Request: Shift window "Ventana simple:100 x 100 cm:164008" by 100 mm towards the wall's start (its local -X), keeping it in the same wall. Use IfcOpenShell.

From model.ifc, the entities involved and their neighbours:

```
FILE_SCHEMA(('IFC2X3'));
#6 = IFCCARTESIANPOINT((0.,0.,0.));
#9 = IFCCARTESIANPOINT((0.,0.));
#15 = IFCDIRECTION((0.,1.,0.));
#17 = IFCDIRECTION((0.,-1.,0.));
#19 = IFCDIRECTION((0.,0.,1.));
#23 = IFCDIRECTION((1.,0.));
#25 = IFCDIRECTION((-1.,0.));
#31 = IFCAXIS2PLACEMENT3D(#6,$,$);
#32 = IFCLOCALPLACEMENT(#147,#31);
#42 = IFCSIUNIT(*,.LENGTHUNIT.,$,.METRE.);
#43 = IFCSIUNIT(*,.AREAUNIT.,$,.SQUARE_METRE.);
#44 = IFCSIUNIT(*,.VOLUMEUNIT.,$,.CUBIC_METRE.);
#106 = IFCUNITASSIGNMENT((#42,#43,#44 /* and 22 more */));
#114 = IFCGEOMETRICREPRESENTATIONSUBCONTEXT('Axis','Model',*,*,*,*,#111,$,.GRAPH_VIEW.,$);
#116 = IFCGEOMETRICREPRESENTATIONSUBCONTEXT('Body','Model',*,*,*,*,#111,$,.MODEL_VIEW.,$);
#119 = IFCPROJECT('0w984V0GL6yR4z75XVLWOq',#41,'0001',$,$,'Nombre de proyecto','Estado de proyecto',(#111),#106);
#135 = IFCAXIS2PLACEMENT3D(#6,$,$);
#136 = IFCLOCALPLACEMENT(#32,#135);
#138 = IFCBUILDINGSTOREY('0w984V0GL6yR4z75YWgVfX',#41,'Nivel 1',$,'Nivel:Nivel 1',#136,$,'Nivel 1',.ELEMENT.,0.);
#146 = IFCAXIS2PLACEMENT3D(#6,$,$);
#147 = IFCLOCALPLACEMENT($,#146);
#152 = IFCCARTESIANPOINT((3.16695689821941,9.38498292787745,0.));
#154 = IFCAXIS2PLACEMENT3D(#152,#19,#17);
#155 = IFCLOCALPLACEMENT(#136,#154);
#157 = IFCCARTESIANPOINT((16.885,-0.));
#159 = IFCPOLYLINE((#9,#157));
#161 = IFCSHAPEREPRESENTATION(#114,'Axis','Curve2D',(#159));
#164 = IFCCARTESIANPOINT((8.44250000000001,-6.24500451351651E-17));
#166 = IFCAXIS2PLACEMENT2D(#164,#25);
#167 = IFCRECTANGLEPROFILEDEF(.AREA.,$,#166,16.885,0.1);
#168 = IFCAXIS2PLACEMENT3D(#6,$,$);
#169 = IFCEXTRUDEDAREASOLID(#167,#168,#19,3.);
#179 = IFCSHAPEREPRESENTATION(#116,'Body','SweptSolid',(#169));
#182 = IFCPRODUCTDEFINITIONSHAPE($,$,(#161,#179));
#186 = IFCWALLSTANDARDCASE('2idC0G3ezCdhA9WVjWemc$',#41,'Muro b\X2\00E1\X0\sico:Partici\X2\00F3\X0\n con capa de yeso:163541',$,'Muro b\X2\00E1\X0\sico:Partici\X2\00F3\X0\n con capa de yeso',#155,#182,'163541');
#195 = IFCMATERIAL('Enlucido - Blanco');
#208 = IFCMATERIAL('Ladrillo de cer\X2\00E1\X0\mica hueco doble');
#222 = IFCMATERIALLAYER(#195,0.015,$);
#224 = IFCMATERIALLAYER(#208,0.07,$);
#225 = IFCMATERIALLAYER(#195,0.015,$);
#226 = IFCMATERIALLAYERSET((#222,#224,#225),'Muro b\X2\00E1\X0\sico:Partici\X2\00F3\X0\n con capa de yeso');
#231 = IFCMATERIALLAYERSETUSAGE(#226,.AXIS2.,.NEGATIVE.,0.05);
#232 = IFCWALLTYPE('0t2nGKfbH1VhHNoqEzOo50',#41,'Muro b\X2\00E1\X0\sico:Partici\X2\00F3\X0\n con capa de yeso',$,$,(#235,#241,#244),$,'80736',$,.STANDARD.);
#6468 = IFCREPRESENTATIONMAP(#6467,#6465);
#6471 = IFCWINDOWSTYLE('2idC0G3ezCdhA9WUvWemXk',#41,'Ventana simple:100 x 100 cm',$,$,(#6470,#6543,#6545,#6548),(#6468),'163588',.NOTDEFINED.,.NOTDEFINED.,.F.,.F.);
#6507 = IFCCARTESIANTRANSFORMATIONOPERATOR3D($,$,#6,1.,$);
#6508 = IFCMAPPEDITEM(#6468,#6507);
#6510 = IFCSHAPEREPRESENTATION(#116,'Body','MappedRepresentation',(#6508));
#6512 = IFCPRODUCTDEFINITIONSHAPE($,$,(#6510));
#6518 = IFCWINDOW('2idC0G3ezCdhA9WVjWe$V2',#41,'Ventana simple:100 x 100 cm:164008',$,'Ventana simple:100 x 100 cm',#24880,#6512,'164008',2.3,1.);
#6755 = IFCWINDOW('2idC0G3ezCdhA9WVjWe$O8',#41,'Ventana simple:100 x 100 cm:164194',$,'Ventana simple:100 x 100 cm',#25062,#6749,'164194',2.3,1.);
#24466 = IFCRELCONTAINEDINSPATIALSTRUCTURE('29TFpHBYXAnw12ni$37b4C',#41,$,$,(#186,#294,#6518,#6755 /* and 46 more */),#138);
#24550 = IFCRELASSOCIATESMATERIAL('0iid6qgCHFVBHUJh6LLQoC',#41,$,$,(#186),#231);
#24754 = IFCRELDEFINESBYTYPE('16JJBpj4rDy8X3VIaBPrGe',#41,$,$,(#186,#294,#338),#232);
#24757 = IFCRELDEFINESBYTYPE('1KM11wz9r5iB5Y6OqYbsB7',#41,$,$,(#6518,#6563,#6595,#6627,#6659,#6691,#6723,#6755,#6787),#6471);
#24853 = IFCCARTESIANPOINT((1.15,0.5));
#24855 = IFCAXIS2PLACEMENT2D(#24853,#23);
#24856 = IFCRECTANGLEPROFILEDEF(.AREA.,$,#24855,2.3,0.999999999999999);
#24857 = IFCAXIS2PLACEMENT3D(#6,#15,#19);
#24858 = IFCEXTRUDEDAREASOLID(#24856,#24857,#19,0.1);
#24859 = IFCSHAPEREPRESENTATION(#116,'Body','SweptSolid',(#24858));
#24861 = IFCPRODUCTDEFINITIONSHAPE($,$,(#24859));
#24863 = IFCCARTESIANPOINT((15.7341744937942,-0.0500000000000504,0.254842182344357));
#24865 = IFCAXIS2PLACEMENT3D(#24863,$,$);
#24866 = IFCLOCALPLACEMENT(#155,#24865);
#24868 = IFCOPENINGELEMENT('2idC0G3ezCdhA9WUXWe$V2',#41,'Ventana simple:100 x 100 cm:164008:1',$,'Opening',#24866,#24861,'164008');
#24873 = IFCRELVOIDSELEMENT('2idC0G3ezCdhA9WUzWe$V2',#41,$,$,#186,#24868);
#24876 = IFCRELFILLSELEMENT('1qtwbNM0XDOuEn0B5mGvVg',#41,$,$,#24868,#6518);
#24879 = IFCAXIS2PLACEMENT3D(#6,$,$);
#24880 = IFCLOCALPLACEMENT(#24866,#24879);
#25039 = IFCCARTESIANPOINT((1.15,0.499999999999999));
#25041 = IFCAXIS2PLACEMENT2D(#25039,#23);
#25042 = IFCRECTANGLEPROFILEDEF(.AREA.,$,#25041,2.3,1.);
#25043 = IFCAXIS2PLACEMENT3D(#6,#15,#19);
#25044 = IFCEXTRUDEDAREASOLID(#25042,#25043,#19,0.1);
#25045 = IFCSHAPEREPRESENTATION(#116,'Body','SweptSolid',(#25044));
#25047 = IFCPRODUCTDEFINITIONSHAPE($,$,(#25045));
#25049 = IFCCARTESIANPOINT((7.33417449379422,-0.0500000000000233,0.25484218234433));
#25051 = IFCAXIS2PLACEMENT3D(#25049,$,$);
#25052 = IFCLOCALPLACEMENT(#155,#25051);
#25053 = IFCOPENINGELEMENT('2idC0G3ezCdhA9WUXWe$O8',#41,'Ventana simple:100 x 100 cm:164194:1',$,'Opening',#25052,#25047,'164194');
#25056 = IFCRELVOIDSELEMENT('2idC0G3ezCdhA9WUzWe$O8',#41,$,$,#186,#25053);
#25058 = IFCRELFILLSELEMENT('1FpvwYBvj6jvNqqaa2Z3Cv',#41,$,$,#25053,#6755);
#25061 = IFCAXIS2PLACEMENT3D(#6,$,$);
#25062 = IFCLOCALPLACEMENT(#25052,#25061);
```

```python
import ifcopenshell
import ifcopenshell.api.geometry
import ifcopenshell.util.placement

model = ifcopenshell.open("model.ifc")

window = model.by_guid("2idC0G3ezCdhA9WVjWe$V2")
opening = window.FillsVoids[0].RelatingOpeningElement
wall = opening.VoidsElements[0].RelatingBuildingElement

wall_matrix = ifcopenshell.util.placement.get_local_placement(wall.ObjectPlacement)
shift = wall_matrix[:3, 0] * -0.1
before = ifcopenshell.util.placement.get_local_placement(window.ObjectPlacement)[:3, 3].copy()

# The window is placed relative to its opening, so it follows when the opening moves.
matrix = ifcopenshell.util.placement.get_local_placement(opening.ObjectPlacement)
matrix[:3, 3] += shift
ifcopenshell.api.geometry.edit_object_placement(
    model, product=opening, matrix=matrix, is_si=False, should_transform_children=True
)

after = ifcopenshell.util.placement.get_local_placement(window.ObjectPlacement)[:3, 3]
print("window moved by", (after - before).round(3) + 0.0)

model.write("model_v2.ifc")
```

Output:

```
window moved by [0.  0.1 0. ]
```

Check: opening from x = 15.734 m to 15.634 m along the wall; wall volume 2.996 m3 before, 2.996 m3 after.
